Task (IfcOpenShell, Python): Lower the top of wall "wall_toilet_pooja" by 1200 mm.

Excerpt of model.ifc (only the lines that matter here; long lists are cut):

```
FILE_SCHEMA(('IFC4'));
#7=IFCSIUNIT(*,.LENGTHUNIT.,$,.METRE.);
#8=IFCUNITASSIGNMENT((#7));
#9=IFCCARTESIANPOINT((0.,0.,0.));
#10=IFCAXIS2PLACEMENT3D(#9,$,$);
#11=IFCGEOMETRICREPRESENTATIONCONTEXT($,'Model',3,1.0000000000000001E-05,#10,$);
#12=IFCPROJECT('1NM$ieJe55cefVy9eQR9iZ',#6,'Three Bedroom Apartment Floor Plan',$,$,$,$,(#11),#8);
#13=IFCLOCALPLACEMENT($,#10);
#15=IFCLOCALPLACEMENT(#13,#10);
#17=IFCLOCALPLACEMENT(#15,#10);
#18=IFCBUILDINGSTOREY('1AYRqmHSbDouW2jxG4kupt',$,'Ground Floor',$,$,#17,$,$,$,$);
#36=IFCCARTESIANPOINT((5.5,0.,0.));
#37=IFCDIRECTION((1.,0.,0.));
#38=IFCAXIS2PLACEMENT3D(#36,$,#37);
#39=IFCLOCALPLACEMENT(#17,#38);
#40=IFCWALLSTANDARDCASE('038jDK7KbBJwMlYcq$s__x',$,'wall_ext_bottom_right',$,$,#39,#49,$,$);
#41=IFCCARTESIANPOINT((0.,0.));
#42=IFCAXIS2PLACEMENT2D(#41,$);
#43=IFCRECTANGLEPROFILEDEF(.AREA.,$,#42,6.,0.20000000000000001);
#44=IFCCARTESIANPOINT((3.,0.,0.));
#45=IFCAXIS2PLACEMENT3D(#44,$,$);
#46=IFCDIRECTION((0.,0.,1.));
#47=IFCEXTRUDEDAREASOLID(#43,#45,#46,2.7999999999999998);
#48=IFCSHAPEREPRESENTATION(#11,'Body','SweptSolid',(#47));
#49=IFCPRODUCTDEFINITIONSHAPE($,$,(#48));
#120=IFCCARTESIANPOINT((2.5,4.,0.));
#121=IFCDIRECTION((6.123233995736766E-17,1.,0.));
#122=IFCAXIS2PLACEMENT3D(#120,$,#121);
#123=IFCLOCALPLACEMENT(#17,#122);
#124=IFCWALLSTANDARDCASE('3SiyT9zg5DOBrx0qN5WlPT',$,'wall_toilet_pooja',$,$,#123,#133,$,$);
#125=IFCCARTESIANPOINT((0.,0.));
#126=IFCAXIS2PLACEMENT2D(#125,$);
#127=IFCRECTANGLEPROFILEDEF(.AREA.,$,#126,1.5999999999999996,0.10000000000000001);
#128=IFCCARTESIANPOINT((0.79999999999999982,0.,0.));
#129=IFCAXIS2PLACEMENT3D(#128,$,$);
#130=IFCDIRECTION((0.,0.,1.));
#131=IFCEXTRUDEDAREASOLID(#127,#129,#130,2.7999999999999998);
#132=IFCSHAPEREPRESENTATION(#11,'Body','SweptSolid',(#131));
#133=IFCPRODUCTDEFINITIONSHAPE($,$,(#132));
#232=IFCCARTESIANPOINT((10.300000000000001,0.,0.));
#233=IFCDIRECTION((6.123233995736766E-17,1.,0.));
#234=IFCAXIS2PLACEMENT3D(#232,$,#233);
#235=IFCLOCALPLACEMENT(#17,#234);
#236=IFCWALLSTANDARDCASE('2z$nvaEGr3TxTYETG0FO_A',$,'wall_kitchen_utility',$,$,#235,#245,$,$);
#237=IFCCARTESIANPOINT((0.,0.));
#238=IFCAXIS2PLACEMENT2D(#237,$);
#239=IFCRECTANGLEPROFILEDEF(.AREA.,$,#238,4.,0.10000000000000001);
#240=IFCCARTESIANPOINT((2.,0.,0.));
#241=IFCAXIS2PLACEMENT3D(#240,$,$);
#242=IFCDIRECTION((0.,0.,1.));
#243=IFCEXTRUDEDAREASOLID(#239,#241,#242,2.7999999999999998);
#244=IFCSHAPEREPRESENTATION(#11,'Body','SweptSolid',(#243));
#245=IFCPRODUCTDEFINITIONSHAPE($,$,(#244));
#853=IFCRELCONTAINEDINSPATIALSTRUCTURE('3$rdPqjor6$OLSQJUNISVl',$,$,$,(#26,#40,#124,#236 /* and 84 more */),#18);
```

```python
import ifcopenshell
import ifcopenshell.geom
import ifcopenshell.util.shape
import ifcopenshell.util.unit

model = ifcopenshell.open("model.ifc")
unit_scale = ifcopenshell.util.unit.calculate_unit_scale(model)
settings = ifcopenshell.geom.settings()


def volume(element):
    """Net volume in cubic metres, openings subtracted."""
    shape = ifcopenshell.geom.create_shape(settings, element)
    return ifcopenshell.util.shape.get_volume(shape.geometry)


wall = model.by_id(124)
before = volume(wall)

body = next(r for r in wall.Representation.Representations if r.RepresentationIdentifier == "Body")
solid = body.Items[0]
old_height = solid.Depth
solid.Depth -= 1.2 / unit_scale
after = volume(wall)

print(f"height {old_height:g} -> {solid.Depth:g}, volume {before:.3f} -> {after:.3f} m3")

model.write("model_rev.ifc")
```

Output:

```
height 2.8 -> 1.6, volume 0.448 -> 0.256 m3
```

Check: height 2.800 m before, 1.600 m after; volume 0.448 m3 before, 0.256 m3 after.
